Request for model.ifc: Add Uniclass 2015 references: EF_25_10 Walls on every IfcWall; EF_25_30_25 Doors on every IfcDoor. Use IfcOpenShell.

First a look at what the model holds.

```python
import ifcopenshell

model = ifcopenshell.open("model.ifc")
print(model.schema)
print("classifications:", [c.Name for c in model.by_type("IfcClassification")])
for ifc_class in ("IfcDoor", "IfcRoof", "IfcStair", "IfcWall", "IfcWindow"):
    print(ifc_class, len(model.by_type(ifc_class)))
```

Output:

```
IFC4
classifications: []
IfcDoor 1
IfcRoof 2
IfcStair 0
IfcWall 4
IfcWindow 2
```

```python
import ifcopenshell
import ifcopenshell.api.classification

model = ifcopenshell.open("model.ifc")

system = ifcopenshell.api.classification.add_classification(model, classification="Uniclass 2015")

codes = {
    "IfcWall": ("EF_25_10", "Walls"),
    "IfcDoor": ("EF_25_30_25", "Doors"),
}
for ifc_class, (code, name) in codes.items():
    products = model.by_type(ifc_class)
    ifcopenshell.api.classification.add_reference(
        model, products=products, classification=system, identification=code, name=name
    )
    print(code, len(products))

model.write("model_rev.ifc")
```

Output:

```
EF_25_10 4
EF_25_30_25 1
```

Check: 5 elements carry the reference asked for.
